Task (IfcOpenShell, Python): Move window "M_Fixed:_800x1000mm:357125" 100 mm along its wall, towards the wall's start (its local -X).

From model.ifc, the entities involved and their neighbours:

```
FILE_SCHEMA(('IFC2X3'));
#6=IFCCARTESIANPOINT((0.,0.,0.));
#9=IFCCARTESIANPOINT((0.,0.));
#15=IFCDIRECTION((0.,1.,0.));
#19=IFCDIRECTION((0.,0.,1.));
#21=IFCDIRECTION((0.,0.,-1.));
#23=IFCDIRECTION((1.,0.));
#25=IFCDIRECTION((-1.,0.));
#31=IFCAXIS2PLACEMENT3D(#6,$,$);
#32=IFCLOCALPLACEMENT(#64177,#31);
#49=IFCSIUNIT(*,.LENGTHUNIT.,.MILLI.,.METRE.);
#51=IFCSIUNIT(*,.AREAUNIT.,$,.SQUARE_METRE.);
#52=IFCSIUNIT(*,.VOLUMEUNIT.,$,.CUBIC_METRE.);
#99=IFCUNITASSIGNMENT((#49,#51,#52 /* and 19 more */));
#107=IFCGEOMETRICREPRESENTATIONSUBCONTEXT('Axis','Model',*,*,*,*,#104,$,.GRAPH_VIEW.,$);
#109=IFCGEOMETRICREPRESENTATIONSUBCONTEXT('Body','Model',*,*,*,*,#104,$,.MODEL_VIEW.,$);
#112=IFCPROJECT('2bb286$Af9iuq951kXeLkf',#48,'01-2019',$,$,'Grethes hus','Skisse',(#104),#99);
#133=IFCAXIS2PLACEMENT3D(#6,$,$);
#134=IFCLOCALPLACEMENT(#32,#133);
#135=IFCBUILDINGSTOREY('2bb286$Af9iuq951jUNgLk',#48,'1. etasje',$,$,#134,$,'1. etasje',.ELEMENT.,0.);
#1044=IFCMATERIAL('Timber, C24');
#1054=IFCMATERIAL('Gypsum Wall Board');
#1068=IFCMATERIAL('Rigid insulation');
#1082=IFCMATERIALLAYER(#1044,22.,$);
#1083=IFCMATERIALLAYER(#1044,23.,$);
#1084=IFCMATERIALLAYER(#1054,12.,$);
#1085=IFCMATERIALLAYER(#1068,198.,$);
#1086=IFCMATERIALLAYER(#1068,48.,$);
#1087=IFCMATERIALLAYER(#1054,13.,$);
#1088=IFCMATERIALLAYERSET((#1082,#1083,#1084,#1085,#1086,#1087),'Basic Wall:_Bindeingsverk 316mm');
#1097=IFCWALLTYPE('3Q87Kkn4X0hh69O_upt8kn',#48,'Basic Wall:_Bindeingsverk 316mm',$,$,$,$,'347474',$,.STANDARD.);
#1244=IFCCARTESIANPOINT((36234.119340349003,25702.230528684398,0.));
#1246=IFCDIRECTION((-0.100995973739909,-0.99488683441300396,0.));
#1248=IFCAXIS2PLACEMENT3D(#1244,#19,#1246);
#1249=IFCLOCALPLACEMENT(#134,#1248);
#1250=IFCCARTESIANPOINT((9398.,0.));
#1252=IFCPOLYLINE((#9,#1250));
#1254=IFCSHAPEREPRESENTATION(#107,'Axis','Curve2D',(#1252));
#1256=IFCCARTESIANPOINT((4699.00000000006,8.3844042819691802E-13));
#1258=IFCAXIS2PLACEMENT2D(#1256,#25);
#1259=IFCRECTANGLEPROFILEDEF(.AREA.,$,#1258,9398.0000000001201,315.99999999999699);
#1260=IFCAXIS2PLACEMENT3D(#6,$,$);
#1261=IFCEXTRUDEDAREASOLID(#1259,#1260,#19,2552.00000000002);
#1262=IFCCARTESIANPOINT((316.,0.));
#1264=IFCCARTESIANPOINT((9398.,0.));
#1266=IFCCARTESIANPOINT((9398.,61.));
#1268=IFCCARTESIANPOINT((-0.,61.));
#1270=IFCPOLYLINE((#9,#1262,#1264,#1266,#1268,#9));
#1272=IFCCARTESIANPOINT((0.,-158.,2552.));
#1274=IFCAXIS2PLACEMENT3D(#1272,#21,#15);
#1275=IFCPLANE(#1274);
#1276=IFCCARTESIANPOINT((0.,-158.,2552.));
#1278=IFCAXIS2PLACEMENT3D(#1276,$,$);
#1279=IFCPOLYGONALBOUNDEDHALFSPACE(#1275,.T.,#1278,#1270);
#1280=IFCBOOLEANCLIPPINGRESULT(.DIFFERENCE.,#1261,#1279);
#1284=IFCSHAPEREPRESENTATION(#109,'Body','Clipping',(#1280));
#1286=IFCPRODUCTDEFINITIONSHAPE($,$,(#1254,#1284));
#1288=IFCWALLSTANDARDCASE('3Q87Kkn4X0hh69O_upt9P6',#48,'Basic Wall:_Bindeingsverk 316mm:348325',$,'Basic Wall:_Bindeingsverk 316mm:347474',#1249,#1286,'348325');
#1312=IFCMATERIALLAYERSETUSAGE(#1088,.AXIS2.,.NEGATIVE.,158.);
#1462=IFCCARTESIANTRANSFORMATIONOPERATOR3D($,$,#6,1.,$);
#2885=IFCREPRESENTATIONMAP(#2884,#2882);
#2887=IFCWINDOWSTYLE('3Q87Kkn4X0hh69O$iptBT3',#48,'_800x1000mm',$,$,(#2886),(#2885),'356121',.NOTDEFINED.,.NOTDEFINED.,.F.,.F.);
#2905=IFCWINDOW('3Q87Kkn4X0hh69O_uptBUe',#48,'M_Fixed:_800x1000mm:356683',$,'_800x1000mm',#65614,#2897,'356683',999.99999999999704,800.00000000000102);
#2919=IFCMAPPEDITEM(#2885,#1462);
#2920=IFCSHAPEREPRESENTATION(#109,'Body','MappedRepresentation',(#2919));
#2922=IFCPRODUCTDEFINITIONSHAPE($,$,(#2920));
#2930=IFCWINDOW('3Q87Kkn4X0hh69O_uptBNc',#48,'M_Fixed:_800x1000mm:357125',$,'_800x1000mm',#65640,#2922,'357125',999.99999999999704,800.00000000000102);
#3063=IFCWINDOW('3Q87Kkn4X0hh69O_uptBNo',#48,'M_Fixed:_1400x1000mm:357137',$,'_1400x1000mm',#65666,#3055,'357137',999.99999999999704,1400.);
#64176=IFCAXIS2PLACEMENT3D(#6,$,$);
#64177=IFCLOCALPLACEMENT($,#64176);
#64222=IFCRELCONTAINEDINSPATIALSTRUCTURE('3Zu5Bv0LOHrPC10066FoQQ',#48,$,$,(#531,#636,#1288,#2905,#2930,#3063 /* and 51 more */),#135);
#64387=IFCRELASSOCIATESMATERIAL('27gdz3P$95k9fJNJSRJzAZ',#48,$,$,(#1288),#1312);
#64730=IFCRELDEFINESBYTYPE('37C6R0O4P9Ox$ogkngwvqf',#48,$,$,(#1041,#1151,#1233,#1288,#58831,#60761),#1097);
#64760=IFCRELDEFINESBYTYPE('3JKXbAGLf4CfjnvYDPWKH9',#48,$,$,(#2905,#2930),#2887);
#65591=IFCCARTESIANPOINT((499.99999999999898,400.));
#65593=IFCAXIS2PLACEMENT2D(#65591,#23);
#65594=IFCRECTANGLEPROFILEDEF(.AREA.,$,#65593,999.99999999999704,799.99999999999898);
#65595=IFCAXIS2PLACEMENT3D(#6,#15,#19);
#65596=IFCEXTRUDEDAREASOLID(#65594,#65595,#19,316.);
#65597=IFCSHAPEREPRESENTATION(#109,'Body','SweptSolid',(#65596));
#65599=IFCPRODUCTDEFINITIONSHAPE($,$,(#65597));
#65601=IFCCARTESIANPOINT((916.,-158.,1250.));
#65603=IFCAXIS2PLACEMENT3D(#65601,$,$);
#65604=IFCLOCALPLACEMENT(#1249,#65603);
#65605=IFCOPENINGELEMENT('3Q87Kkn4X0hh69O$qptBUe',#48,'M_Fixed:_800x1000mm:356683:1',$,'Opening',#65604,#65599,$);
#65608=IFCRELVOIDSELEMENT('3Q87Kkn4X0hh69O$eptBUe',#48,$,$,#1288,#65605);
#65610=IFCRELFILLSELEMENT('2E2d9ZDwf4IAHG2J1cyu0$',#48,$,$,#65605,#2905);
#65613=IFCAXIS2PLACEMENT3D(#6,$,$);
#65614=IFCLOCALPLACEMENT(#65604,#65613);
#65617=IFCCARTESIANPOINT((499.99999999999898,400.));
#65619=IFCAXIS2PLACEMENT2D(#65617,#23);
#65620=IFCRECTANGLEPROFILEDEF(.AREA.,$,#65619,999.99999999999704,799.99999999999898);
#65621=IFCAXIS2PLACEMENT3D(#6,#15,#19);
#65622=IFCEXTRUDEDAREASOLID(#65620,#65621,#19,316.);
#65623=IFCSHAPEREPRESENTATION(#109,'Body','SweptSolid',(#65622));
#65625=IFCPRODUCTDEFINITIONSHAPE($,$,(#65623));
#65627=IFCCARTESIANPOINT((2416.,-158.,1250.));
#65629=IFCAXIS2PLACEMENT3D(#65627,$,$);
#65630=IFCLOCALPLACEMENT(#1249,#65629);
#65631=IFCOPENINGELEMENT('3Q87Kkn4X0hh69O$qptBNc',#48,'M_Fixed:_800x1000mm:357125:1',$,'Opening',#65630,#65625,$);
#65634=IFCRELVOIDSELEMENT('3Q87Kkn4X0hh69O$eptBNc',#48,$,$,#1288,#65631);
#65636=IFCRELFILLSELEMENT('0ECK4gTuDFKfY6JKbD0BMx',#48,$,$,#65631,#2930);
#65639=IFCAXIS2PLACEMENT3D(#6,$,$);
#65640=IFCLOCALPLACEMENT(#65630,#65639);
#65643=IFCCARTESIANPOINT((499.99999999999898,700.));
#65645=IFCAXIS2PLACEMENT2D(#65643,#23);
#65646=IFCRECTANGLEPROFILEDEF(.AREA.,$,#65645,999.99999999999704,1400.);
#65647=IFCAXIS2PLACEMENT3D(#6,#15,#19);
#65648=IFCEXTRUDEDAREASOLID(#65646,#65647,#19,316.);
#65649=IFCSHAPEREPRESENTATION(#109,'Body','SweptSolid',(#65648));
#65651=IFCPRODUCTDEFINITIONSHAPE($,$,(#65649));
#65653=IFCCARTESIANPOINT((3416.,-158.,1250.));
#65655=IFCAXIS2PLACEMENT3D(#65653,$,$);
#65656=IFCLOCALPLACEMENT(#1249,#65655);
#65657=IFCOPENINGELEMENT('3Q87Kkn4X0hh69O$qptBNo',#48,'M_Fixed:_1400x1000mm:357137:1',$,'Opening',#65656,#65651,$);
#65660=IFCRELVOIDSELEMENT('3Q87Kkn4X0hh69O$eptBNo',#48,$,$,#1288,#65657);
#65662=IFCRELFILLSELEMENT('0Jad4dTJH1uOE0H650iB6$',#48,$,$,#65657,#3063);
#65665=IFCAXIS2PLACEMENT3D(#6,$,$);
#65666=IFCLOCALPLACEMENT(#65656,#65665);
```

```python
import ifcopenshell
import ifcopenshell.api.geometry
import ifcopenshell.util.placement
import ifcopenshell.util.unit

model = ifcopenshell.open("model.ifc")
unit_scale = ifcopenshell.util.unit.calculate_unit_scale(model)

window = model.by_guid("3Q87Kkn4X0hh69O_uptBNc")
opening = window.FillsVoids[0].RelatingOpeningElement
wall = opening.VoidsElements[0].RelatingBuildingElement

wall_matrix = ifcopenshell.util.placement.get_local_placement(wall.ObjectPlacement)
shift = wall_matrix[:3, 0] * -0.1 / unit_scale
before = ifcopenshell.util.placement.get_local_placement(window.ObjectPlacement)[:3, 3].copy()

# The window is placed relative to its opening, so it follows when the opening moves.
matrix = ifcopenshell.util.placement.get_local_placement(opening.ObjectPlacement)
matrix[:3, 3] += shift
ifcopenshell.api.geometry.edit_object_placement(
    model, product=opening, matrix=matrix, is_si=False, should_transform_children=True
)

after = ifcopenshell.util.placement.get_local_placement(window.ObjectPlacement)[:3, 3]
print("window moved by", (after - before).round(3) + 0.0)

model.write("model_rev.ifc")
```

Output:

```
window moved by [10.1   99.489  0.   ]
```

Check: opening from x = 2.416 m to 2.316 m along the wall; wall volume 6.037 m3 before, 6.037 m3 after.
